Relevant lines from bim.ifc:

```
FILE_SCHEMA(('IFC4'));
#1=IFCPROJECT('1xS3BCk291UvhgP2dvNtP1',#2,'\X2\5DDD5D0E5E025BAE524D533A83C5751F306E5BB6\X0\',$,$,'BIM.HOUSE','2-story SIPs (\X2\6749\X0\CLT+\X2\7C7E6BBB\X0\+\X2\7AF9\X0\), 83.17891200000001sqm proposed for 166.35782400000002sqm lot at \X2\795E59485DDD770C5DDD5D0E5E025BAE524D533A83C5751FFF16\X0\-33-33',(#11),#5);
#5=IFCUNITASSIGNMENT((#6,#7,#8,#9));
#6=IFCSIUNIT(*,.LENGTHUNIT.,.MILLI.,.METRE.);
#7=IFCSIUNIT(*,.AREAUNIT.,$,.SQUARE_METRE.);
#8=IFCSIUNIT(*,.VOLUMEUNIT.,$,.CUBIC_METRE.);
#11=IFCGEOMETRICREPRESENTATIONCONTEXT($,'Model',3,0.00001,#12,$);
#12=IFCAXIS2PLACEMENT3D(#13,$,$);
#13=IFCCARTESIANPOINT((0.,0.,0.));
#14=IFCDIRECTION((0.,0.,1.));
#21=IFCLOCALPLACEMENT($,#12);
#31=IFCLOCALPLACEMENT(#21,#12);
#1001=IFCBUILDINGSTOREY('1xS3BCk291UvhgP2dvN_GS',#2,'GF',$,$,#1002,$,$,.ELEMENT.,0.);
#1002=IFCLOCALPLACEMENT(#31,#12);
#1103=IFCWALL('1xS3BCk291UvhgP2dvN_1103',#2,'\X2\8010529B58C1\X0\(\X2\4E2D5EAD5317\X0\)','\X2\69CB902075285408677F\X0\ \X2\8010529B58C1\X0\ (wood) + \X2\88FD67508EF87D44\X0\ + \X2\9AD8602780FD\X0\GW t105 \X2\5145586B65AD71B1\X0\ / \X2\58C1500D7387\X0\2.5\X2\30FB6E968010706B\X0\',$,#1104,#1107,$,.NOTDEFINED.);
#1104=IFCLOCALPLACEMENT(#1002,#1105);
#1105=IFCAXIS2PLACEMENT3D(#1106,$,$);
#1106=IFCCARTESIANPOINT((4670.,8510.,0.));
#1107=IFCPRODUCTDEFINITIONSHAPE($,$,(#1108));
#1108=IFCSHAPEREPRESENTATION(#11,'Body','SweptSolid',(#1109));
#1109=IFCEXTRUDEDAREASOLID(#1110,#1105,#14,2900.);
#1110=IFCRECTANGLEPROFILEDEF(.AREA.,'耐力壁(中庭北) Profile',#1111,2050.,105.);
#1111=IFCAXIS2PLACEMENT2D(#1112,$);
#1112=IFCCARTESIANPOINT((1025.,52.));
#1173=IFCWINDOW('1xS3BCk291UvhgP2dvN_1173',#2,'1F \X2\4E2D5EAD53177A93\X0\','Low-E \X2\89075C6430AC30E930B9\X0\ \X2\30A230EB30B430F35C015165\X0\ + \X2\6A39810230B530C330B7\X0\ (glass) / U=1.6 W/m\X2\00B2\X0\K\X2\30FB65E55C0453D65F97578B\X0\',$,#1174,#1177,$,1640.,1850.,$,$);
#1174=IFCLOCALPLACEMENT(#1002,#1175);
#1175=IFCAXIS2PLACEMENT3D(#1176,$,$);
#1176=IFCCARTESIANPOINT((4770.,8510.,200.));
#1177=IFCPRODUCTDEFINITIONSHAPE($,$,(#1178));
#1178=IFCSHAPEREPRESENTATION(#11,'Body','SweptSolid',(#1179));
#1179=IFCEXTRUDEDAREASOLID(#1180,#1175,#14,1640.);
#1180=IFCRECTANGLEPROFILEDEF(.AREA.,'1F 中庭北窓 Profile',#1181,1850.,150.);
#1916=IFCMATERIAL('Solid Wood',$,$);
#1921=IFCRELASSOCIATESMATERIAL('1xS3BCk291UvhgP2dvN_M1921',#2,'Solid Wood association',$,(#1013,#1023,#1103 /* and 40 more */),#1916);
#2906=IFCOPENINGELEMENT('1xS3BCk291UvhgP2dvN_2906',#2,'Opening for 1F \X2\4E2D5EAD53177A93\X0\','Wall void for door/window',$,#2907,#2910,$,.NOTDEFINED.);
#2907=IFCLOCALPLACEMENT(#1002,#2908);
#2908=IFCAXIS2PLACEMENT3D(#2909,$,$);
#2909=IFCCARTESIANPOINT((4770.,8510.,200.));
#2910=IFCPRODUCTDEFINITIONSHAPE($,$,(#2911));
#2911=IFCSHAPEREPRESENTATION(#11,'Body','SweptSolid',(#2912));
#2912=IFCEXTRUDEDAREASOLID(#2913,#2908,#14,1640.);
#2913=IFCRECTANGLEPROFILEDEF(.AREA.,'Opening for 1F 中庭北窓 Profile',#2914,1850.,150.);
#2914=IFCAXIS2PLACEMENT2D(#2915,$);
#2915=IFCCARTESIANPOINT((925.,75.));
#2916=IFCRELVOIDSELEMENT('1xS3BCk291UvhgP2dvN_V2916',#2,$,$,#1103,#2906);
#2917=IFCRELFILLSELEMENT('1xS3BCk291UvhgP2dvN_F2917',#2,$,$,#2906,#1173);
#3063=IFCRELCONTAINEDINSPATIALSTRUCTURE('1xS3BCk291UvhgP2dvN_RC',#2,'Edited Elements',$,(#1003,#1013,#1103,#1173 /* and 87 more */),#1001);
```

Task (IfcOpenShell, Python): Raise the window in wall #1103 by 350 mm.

```python
import numpy as np
import ifcopenshell
import ifcopenshell.api.geometry
import ifcopenshell.util.placement
import ifcopenshell.util.unit

model = ifcopenshell.open("bim.ifc")
unit_scale = ifcopenshell.util.unit.calculate_unit_scale(model)

window = model.by_guid("1xS3BCk291UvhgP2dvN_1173")
opening = window.FillsVoids[0].RelatingOpeningElement
dz = 0.35 / unit_scale

shift = np.array([0.0, 0.0, dz])
# The window is not placed relative to its opening, so move both.
for product in (opening, window):
    matrix = ifcopenshell.util.placement.get_local_placement(product.ObjectPlacement)
    matrix[:3, 3] += shift
    ifcopenshell.api.geometry.edit_object_placement(model, product=product, matrix=matrix, is_si=False)

print(f"moved by {dz * unit_scale:+.3f} m")

model.write("bim_edited.ifc")
```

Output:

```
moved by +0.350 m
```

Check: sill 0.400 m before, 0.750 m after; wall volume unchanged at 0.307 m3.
